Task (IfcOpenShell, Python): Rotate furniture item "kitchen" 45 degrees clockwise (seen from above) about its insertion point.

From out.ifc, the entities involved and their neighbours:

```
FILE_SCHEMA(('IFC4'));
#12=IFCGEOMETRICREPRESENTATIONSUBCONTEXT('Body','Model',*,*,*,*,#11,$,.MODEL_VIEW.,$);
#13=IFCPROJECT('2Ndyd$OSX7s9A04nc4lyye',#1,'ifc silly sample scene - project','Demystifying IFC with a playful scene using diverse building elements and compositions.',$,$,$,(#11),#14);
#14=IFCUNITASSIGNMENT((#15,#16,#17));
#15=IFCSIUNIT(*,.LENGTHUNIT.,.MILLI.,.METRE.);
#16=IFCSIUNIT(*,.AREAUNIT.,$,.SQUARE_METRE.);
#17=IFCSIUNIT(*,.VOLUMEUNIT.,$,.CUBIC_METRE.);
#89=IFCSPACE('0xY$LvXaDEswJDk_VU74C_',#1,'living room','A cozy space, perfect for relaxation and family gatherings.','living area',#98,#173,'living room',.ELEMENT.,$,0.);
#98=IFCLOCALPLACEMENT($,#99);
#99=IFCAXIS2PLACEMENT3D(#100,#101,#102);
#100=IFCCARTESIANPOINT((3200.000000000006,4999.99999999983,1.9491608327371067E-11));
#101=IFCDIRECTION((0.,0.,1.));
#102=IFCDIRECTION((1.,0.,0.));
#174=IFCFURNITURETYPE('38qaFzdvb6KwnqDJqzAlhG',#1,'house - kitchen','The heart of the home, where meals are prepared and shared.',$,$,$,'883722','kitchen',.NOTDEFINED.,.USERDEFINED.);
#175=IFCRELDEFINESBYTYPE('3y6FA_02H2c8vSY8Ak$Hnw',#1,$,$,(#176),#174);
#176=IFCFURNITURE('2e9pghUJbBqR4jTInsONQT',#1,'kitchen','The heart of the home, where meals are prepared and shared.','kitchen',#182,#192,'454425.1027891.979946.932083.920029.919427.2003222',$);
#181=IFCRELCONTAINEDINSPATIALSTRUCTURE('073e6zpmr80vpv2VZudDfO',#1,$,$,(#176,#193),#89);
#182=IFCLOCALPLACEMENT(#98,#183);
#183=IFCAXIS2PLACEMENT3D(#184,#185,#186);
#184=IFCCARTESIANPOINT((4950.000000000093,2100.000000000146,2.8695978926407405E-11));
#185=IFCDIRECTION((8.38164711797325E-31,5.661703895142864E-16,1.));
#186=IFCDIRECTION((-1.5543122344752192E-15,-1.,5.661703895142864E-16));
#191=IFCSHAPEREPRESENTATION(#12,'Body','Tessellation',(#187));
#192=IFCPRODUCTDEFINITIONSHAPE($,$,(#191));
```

```python
import ifcopenshell
import ifcopenshell.api.geometry
import ifcopenshell.util.placement

model = ifcopenshell.open("out.ifc")

item = model.by_guid("2e9pghUJbBqR4jTInsONQT")
matrix = ifcopenshell.util.placement.get_local_placement(item.ObjectPlacement)
matrix = matrix @ ifcopenshell.util.placement.rotation(-45, "Z")
ifcopenshell.api.geometry.edit_object_placement(model, product=item, matrix=matrix, is_si=False)

print(ifcopenshell.util.placement.get_local_placement(item.ObjectPlacement).round(3) + 0.0)

model.write("out_updated.ifc")
```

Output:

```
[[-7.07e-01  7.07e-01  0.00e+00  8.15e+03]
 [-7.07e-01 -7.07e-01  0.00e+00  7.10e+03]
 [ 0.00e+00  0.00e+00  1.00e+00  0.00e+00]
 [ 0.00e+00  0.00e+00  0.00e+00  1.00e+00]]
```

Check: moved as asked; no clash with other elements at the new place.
